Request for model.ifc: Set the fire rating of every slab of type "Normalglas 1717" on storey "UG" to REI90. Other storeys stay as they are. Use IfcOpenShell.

First a look at what the model holds.

```python
import ifcopenshell
import ifcopenshell.util.element

model = ifcopenshell.open("model.ifc")
print(model.schema)
storey = next(s for s in model.by_type("IfcBuildingStorey") if s.Name == "UG")
slabs = [e for e in ifcopenshell.util.element.get_decomposition(storey) if e.is_a("IfcSlab")]
seen = {}
for e in slabs:
    element_type = ifcopenshell.util.element.get_type(e)
    key = (element_type.Name if element_type != e and element_type else None, ifcopenshell.util.element.get_pset(e, "Pset_SlabCommon", "FireRating"))
    seen[key] = seen.get(key, 0) + 1
for (name, value), count in sorted(seen.items(), key=str):
    print(count, "x", name, "|", value)
```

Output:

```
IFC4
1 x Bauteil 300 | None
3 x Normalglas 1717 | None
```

```python
import ifcopenshell
import ifcopenshell.api.pset
import ifcopenshell.util.element

model = ifcopenshell.open("model.ifc")

storey = next(s for s in model.by_type("IfcBuildingStorey") if s.Name == "UG")
slabs = [e for e in ifcopenshell.util.element.get_decomposition(storey) if e.is_a("IfcSlab")]

count = 0
for e in slabs:
    element_type = ifcopenshell.util.element.get_type(e)
    if element_type in (None, e) or element_type.Name != "Normalglas 1717":
        continue
    # add_pset returns the element's existing set when there is one.
    pset = ifcopenshell.api.pset.add_pset(model, product=e, name="Pset_SlabCommon")
    ifcopenshell.api.pset.edit_pset(model, pset=pset, properties={"FireRating": "REI90"})
    count += 1

print(count, "slabs updated")

model.write("model_updated.ifc")
```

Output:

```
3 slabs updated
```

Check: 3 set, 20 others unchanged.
